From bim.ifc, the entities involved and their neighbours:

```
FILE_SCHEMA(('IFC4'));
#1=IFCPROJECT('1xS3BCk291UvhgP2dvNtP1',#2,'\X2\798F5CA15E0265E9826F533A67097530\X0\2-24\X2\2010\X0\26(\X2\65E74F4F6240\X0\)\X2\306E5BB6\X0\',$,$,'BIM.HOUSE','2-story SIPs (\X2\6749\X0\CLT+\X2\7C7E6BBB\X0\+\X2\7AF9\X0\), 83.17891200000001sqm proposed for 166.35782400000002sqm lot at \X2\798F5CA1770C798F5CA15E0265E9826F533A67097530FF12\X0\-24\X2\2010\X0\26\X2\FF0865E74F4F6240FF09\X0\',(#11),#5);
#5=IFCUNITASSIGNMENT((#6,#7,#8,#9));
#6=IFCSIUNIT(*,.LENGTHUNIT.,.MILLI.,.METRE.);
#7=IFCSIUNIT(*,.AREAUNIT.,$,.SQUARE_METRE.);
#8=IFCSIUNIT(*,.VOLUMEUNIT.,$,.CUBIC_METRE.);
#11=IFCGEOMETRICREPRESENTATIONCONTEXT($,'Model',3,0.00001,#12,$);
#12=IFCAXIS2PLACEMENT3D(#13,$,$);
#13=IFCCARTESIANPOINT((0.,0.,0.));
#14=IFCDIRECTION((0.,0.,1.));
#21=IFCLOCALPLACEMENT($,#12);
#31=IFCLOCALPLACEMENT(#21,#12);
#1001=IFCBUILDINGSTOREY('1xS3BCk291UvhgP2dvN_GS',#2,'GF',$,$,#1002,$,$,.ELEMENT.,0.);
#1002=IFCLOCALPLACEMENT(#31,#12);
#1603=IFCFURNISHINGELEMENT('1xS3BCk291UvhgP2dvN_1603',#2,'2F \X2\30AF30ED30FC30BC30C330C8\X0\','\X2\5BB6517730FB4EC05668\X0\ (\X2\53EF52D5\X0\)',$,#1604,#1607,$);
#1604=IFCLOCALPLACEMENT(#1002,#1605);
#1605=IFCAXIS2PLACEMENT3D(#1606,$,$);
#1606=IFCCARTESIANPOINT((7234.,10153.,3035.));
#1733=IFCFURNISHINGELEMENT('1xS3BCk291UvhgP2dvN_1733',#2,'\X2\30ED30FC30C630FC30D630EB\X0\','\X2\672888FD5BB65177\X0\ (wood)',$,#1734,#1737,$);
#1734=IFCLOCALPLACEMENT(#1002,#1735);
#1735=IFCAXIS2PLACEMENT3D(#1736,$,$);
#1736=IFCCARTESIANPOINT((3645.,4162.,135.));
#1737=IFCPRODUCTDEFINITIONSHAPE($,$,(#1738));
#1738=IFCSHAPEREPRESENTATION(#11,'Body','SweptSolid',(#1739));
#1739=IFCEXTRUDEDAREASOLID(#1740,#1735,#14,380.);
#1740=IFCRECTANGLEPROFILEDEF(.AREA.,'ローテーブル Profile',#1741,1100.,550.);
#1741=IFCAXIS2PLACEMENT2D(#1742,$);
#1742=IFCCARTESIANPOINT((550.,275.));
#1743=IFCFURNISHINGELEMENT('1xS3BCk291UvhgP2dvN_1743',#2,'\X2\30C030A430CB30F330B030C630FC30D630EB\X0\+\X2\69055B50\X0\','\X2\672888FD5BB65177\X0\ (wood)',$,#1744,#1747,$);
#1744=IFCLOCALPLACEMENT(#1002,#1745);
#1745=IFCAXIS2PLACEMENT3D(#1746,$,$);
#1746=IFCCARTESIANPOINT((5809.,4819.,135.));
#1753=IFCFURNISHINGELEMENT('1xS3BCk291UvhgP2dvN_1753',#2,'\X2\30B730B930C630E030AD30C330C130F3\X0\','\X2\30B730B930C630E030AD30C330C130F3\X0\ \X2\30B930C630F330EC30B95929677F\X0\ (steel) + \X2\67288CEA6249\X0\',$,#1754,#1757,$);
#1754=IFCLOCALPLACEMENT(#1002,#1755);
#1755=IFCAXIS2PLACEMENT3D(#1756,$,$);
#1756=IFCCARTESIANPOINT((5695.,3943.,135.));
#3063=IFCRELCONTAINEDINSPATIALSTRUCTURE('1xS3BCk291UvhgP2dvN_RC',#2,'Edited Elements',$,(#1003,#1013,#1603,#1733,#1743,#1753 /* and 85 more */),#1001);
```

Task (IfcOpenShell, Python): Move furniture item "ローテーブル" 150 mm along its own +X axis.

```python
import ifcopenshell
import ifcopenshell.api.geometry
import ifcopenshell.util.placement
import ifcopenshell.util.unit

model = ifcopenshell.open("bim.ifc")
unit_scale = ifcopenshell.util.unit.calculate_unit_scale(model)

item = model.by_guid("1xS3BCk291UvhgP2dvN_1733")
matrix = ifcopenshell.util.placement.get_local_placement(item.ObjectPlacement)
matrix[:3, 3] += matrix[:3, 0] * 0.15 / unit_scale
ifcopenshell.api.geometry.edit_object_placement(model, product=item, matrix=matrix, is_si=False)

print(ifcopenshell.util.placement.get_local_placement(item.ObjectPlacement).round(3) + 0.0)

model.write("bim_updated.ifc")
```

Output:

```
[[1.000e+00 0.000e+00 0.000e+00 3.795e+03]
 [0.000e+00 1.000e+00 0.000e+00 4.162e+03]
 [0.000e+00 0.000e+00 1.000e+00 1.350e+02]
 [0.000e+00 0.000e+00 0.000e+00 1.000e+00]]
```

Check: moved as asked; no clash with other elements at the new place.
